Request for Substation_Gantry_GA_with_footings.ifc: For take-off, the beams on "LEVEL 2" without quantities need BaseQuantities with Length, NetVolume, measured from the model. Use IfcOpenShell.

First a look at what the model holds.

```python
import ifcopenshell
import ifcopenshell.util.element
import ifcopenshell.util.unit

model = ifcopenshell.open("Substation_Gantry_GA_with_footings.ifc")
print(model.schema)
for unit_type in ("LENGTHUNIT", "AREAUNIT", "VOLUMEUNIT"):
    print(unit_type, ifcopenshell.util.unit.calculate_unit_scale(model, unit_type))
storey = next(s for s in model.by_type("IfcBuildingStorey") if s.Name == "LEVEL 2")
beams = [e for e in ifcopenshell.util.element.get_decomposition(storey) if e.is_a("IfcBeam")]
for e in sorted(beams, key=lambda e: e.id()):
    print(e.id(), e.is_a(), e.Name, list(ifcopenshell.util.element.get_psets(e, qtos_only=True)), sep=" | ")
```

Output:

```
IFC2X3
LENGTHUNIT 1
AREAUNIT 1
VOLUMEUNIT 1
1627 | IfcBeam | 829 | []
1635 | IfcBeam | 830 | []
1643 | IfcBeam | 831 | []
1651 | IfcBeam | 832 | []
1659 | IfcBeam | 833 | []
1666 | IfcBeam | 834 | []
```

```python
import ifcopenshell
import ifcopenshell.api.pset
import ifcopenshell.geom
import ifcopenshell.util.element
import ifcopenshell.util.shape
import ifcopenshell.util.unit

model = ifcopenshell.open("Substation_Gantry_GA_with_footings.ifc")
unit_scale = ifcopenshell.util.unit.calculate_unit_scale(model)
volume_scale = ifcopenshell.util.unit.calculate_unit_scale(model, "VOLUMEUNIT")
settings = ifcopenshell.geom.settings()

storey = next(s for s in model.by_type("IfcBuildingStorey") if s.Name == "LEVEL 2")
beams = [e for e in ifcopenshell.util.element.get_decomposition(storey) if e.is_a("IfcBeam")]

for e in sorted(beams, key=lambda e: e.id()):
    if ifcopenshell.util.element.get_psets(e, qtos_only=True, should_inherit=False):
        continue
    # Geometry comes back in metres, in the element's own axes.
    shape = ifcopenshell.geom.create_shape(settings, e)
    values = {
        "Length": ifcopenshell.util.shape.get_max_xyz(shape.geometry) / unit_scale,
        "NetVolume": ifcopenshell.util.shape.get_volume(shape.geometry) / volume_scale,
    }
    qto = ifcopenshell.api.pset.add_qto(model, product=e, name="BaseQuantities")
    ifcopenshell.api.pset.edit_qto(model, qto=qto, properties=values)
    print(e.id(), {k: round(v, 3) for k, v in values.items()})

model.write("Substation_Gantry_GA_with_footings_v2.ifc")
```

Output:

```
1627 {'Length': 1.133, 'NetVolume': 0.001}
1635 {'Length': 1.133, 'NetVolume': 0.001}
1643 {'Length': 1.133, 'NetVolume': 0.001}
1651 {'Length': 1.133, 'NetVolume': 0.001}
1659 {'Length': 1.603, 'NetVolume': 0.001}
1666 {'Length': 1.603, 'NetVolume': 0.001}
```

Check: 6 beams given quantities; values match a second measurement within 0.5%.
